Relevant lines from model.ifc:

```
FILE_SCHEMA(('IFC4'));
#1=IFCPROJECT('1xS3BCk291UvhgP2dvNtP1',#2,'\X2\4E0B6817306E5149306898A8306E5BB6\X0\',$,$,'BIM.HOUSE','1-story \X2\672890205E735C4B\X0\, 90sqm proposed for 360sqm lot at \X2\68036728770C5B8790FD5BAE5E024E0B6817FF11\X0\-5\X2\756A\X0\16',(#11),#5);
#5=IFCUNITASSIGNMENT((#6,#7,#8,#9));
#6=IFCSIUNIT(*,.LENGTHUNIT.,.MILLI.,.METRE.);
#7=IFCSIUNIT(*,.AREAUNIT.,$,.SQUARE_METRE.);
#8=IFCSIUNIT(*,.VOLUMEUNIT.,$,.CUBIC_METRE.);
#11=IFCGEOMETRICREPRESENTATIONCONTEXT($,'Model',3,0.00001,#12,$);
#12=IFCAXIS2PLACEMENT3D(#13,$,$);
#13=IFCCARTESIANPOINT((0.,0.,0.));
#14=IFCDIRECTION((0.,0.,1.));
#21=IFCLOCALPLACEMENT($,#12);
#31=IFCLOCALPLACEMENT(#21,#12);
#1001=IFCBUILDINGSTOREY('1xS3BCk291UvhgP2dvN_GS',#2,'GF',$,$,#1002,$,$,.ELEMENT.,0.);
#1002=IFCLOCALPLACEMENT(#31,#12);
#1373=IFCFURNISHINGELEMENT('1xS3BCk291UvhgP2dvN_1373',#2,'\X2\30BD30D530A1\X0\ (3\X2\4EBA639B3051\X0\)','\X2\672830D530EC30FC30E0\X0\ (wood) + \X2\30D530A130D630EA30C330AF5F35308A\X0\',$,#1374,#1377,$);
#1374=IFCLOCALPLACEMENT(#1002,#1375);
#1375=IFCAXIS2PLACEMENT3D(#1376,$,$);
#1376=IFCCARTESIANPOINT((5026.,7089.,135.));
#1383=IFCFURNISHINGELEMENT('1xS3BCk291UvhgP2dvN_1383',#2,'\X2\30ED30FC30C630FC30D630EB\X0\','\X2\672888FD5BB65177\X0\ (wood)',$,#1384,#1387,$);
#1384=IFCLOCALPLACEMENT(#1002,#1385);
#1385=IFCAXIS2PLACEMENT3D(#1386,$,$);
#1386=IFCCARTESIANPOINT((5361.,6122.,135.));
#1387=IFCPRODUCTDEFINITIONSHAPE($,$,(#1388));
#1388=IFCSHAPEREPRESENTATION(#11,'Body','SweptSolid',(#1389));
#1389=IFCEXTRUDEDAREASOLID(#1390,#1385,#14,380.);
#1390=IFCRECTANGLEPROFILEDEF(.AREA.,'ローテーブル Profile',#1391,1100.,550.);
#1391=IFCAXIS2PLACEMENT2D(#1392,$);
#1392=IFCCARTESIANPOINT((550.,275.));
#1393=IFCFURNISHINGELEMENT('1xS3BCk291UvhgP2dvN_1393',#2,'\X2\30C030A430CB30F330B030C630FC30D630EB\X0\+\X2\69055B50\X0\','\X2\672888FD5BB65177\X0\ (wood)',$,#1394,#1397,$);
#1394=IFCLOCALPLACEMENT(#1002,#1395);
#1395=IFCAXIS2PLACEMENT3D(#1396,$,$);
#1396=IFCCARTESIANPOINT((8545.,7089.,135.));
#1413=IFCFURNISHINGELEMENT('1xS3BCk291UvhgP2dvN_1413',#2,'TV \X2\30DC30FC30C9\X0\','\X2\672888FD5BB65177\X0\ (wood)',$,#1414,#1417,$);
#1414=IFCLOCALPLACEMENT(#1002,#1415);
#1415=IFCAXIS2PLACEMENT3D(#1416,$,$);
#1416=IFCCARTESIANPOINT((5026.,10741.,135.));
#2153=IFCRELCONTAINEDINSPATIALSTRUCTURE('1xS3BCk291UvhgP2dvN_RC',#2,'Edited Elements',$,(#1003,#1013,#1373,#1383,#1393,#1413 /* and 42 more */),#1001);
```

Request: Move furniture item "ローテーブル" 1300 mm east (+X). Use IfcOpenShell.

```python
import ifcopenshell
import ifcopenshell.api.geometry
import ifcopenshell.util.placement
import ifcopenshell.util.unit

model = ifcopenshell.open("model.ifc")
unit_scale = ifcopenshell.util.unit.calculate_unit_scale(model)

item = model.by_id(1383)
matrix = ifcopenshell.util.placement.get_local_placement(item.ObjectPlacement)
matrix[0, 3] += 1.3 / unit_scale
ifcopenshell.api.geometry.edit_object_placement(model, product=item, matrix=matrix, is_si=False)

print(ifcopenshell.util.placement.get_local_placement(item.ObjectPlacement).round(3) + 0.0)

model.write("model_edited.ifc")
```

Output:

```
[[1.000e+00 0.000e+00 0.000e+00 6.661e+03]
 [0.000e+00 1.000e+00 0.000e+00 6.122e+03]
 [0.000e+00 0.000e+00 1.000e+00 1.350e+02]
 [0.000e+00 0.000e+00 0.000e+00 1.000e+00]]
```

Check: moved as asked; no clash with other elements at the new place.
